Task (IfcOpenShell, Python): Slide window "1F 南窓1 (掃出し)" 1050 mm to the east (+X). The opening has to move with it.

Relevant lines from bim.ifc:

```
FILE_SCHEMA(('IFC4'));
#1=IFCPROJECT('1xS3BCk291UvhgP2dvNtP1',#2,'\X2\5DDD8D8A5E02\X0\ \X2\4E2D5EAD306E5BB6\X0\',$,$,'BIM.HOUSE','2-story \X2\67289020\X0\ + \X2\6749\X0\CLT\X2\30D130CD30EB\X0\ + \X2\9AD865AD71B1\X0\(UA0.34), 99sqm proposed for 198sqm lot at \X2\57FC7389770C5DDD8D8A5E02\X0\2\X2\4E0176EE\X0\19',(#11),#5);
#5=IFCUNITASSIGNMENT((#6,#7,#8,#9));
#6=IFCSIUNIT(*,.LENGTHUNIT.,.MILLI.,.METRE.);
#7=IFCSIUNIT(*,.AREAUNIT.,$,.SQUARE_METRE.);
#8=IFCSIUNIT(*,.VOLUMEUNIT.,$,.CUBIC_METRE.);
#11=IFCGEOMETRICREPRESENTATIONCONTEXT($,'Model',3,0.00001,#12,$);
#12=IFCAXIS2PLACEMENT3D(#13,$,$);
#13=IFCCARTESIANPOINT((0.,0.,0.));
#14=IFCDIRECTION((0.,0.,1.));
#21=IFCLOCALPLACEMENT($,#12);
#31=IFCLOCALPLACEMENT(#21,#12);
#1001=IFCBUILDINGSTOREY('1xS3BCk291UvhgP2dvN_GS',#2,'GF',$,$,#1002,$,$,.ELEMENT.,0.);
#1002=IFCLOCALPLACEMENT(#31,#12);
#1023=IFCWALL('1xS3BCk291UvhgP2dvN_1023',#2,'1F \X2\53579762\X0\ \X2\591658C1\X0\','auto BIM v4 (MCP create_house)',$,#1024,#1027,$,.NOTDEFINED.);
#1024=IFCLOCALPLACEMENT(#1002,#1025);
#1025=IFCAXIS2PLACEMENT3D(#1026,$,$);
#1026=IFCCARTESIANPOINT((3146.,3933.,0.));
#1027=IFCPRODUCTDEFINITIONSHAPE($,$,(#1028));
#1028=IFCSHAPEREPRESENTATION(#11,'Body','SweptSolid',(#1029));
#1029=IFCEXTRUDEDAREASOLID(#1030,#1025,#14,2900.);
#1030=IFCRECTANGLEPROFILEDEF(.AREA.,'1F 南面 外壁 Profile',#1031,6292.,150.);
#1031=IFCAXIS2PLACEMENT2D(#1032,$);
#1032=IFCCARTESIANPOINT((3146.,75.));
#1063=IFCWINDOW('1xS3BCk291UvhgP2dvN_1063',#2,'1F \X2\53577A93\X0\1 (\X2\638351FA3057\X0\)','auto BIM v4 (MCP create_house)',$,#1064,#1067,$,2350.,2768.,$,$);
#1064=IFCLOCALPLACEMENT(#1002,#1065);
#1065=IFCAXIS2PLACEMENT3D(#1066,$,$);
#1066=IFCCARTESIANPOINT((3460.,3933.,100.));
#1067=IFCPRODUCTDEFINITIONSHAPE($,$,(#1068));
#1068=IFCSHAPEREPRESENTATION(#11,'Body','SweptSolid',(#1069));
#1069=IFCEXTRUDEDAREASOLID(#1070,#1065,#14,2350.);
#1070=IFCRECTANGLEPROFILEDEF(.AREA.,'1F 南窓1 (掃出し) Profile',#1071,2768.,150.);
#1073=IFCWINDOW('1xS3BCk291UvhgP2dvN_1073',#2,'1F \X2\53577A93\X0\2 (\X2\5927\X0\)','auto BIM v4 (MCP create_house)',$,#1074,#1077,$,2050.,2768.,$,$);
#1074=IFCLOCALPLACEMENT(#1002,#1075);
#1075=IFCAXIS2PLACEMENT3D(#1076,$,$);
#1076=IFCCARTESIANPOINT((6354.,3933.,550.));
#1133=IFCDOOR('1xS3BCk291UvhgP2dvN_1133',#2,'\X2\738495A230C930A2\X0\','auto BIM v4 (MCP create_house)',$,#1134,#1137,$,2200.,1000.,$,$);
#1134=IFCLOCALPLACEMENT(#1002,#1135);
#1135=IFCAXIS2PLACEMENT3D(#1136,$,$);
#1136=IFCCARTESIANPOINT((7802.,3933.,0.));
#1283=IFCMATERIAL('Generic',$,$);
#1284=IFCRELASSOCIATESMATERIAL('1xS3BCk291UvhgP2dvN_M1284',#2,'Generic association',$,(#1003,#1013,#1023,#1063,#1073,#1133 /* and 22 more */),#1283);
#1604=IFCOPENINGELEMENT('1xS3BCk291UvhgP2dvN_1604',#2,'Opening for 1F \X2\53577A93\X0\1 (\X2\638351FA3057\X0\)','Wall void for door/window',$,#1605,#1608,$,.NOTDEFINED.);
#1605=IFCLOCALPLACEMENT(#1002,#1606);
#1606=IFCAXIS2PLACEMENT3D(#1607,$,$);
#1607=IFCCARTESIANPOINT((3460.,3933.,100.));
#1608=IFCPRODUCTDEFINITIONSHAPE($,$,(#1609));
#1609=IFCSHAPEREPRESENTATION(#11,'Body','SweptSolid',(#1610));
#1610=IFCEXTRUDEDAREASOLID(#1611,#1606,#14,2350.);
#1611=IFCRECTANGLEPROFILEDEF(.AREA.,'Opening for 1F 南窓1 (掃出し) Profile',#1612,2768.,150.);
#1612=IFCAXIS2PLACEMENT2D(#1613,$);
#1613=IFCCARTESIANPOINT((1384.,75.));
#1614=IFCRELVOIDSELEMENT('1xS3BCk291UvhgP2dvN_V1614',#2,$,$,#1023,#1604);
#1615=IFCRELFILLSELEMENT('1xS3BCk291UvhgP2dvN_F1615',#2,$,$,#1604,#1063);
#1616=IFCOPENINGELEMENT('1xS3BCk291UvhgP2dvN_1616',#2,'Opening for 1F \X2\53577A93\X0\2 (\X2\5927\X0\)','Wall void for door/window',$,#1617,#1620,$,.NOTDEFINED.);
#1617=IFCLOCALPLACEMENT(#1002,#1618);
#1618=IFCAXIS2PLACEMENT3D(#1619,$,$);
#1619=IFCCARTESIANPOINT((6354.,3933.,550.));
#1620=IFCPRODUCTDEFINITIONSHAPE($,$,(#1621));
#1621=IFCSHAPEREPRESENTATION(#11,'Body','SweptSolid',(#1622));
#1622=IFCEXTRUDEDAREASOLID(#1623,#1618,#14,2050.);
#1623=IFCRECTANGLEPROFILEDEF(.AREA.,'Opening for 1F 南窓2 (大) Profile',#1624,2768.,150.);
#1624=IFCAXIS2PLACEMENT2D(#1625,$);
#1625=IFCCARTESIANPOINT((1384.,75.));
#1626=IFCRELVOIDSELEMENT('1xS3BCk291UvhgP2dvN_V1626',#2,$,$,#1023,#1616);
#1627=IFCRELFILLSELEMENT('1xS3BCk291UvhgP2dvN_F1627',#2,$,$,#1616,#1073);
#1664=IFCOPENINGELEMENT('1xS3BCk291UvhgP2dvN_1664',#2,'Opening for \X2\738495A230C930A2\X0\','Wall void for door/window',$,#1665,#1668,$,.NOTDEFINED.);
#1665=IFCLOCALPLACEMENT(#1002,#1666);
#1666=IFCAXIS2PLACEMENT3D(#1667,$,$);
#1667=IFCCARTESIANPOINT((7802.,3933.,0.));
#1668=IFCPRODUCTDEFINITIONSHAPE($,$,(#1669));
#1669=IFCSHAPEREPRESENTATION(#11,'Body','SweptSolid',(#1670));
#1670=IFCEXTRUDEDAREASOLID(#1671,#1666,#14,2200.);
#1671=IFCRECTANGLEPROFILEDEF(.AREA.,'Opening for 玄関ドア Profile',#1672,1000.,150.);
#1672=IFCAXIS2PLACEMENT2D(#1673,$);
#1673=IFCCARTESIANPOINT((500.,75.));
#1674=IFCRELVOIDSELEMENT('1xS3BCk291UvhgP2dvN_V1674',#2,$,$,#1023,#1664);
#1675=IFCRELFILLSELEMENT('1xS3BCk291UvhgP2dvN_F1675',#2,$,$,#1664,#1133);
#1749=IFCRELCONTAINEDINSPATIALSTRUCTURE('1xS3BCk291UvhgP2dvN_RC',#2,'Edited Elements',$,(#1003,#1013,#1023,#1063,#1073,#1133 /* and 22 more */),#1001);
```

```python
import ifcopenshell
import ifcopenshell.api.geometry
import ifcopenshell.util.placement

model = ifcopenshell.open("bim.ifc")

window = model.by_id(1063)
opening = window.FillsVoids[0].RelatingOpeningElement
wall = opening.VoidsElements[0].RelatingBuildingElement

wall_matrix = ifcopenshell.util.placement.get_local_placement(wall.ObjectPlacement)
shift = wall_matrix[:3, 0] * 1050.0
before = ifcopenshell.util.placement.get_local_placement(window.ObjectPlacement)[:3, 3].copy()

# The window is not placed relative to its opening, so move both.
for product in (opening, window):
    matrix = ifcopenshell.util.placement.get_local_placement(product.ObjectPlacement)
    matrix[:3, 3] += shift
    ifcopenshell.api.geometry.edit_object_placement(model, product=product, matrix=matrix, is_si=False)

after = ifcopenshell.util.placement.get_local_placement(window.ObjectPlacement)[:3, 3]
print("window moved by", (after - before).round(3) + 0.0)

model.write("bim_rev.ifc")
```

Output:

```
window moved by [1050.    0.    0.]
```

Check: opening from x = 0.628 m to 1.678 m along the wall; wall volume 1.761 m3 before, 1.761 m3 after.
